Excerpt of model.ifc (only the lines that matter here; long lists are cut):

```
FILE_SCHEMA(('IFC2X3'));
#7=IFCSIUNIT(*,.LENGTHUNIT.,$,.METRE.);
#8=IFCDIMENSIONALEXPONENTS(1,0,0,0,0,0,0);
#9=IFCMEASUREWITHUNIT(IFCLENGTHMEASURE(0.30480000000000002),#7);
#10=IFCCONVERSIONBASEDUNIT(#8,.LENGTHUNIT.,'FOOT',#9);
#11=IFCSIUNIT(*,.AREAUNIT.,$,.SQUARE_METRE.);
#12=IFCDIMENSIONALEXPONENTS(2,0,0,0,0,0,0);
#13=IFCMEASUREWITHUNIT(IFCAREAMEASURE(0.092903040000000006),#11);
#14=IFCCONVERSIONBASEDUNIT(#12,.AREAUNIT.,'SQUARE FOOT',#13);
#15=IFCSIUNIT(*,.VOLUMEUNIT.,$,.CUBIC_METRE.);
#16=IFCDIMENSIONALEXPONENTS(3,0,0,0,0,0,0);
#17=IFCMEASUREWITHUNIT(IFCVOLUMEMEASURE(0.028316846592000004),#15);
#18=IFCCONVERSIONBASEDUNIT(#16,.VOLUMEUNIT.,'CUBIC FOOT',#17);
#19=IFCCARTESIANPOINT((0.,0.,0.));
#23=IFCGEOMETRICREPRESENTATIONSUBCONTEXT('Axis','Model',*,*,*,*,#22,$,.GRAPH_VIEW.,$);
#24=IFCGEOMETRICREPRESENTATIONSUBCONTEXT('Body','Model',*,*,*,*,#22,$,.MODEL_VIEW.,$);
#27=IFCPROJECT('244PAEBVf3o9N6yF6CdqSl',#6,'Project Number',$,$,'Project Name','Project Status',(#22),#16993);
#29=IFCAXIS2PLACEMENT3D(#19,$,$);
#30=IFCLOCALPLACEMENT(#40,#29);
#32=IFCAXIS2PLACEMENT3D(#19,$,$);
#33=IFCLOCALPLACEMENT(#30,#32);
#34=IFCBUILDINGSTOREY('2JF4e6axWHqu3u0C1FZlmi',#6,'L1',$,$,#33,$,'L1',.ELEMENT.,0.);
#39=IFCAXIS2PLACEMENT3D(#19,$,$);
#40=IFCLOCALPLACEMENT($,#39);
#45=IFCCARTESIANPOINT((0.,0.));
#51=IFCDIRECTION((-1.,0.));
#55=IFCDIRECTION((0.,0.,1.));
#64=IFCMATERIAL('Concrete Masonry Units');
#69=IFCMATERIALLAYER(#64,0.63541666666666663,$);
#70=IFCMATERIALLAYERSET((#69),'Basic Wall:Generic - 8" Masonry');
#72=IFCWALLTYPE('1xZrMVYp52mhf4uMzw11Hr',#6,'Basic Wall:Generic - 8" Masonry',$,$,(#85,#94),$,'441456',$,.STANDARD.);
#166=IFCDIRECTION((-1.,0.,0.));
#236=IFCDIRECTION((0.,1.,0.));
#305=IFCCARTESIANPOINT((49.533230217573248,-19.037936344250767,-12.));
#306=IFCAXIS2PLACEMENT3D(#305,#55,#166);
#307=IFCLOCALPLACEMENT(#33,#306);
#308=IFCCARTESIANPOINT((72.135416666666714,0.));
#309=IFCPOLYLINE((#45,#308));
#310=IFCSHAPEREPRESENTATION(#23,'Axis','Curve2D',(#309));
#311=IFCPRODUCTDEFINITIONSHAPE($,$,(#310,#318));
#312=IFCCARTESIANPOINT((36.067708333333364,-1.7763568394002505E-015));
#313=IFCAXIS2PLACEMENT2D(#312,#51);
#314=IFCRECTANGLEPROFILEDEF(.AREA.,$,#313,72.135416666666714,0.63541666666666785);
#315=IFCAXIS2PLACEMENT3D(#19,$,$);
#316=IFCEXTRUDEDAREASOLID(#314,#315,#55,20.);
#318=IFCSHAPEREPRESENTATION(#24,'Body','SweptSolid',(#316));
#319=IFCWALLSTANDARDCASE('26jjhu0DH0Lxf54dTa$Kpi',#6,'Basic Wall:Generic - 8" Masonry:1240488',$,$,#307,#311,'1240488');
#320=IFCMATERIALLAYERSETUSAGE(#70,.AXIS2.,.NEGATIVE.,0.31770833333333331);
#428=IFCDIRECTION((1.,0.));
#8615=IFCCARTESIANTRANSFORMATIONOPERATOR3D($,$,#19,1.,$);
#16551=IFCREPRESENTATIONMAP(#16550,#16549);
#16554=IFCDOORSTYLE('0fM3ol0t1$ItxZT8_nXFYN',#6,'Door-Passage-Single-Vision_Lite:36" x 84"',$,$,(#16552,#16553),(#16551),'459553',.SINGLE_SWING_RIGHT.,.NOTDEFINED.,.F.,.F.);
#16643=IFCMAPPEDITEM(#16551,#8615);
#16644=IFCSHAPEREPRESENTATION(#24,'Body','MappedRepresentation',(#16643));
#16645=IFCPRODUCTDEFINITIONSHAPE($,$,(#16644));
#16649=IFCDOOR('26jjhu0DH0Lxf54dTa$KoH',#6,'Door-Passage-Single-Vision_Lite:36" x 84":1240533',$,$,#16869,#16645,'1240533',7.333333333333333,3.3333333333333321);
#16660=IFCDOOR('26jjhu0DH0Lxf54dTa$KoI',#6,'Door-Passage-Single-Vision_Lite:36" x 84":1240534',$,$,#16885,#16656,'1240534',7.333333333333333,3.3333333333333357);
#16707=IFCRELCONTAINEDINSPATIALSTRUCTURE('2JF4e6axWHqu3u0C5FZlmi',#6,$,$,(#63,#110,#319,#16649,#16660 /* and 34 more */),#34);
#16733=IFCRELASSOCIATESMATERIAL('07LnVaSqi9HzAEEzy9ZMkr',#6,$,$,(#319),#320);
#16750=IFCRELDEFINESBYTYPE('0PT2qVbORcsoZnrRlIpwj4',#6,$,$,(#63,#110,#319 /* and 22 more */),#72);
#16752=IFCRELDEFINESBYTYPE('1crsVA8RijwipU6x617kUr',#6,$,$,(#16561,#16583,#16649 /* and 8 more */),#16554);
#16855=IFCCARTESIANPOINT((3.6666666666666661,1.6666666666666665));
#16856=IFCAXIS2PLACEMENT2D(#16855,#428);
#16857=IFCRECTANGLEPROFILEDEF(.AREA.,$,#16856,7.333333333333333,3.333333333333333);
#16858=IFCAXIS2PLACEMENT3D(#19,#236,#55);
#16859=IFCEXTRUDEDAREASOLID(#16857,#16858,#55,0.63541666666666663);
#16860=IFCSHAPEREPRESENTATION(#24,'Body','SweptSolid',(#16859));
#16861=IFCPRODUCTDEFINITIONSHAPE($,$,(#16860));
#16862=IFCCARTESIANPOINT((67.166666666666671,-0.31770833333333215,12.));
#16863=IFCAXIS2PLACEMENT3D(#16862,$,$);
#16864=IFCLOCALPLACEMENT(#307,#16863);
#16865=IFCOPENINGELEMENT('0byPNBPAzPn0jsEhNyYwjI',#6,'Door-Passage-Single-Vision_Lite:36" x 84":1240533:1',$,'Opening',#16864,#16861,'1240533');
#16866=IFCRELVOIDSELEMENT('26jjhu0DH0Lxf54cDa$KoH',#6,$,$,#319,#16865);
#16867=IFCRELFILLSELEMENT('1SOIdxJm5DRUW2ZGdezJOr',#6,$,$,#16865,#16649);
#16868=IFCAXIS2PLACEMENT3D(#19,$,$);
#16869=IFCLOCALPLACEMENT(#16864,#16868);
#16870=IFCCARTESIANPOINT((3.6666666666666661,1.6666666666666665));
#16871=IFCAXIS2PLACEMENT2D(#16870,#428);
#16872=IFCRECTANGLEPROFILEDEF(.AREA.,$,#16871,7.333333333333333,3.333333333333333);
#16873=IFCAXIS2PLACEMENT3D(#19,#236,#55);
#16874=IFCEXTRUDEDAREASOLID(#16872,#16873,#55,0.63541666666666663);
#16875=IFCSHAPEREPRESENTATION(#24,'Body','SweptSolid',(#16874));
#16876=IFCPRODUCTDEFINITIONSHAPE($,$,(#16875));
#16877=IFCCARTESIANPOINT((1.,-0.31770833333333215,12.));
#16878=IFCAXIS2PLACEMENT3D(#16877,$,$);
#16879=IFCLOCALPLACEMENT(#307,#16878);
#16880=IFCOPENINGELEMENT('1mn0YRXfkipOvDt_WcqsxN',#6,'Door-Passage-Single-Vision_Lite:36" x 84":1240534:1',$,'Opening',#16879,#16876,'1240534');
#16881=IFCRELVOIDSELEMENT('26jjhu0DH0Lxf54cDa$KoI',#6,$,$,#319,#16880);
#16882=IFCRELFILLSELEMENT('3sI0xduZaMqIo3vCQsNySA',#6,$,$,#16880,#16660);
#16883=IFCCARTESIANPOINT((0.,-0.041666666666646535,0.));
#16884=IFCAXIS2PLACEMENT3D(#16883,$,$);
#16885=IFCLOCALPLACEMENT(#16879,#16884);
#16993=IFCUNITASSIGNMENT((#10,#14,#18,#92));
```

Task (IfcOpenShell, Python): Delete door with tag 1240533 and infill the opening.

```python
import ifcopenshell
import ifcopenshell.api.feature
import ifcopenshell.api.root
import ifcopenshell.geom
import ifcopenshell.util.shape

model = ifcopenshell.open("model.ifc")
settings = ifcopenshell.geom.settings()


def volume(element):
    """Net volume in cubic metres, openings subtracted."""
    shape = ifcopenshell.geom.create_shape(settings, element)
    return ifcopenshell.util.shape.get_volume(shape.geometry)


door = model.by_id(16649)
opening = door.FillsVoids[0].RelatingOpeningElement
wall = opening.VoidsElements[0].RelatingBuildingElement
before = volume(wall)

ifcopenshell.api.root.remove_product(model, product=door)
ifcopenshell.api.feature.remove_feature(model, feature=opening)

after = volume(wall)

print(f"wall volume {before:.3f} -> {after:.3f} m3")

model.write("model_updated.ifc")
```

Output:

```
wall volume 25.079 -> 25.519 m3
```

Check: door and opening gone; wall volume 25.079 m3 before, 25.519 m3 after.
